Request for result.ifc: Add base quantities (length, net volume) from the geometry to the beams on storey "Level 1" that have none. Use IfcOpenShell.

First a look at what the model holds.

```python
import ifcopenshell
import ifcopenshell.util.element
import ifcopenshell.util.unit

model = ifcopenshell.open("result.ifc")
print(model.schema)
for unit_type in ("LENGTHUNIT", "AREAUNIT", "VOLUMEUNIT"):
    print(unit_type, ifcopenshell.util.unit.calculate_unit_scale(model, unit_type))
storey = next(s for s in model.by_type("IfcBuildingStorey") if s.Name == "Level 1")
beams = [e for e in ifcopenshell.util.element.get_decomposition(storey) if e.is_a("IfcBeam")]
for e in sorted(beams, key=lambda e: e.id()):
    print(e.id(), e.is_a(), e.Name, list(ifcopenshell.util.element.get_psets(e, qtos_only=True)), sep=" | ")
```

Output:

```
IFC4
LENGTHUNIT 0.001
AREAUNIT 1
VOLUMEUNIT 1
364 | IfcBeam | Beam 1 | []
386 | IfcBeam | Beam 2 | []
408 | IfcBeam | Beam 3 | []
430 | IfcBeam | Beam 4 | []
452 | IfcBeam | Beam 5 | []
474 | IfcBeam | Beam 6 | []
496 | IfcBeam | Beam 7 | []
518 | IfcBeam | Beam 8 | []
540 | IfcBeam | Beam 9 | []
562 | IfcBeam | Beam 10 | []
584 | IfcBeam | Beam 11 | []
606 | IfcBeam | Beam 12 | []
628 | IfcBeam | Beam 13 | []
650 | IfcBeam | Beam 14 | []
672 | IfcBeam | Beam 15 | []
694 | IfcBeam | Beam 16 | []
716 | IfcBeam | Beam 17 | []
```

```python
import ifcopenshell
import ifcopenshell.api.pset
import ifcopenshell.geom
import ifcopenshell.util.element
import ifcopenshell.util.shape
import ifcopenshell.util.unit

model = ifcopenshell.open("result.ifc")
unit_scale = ifcopenshell.util.unit.calculate_unit_scale(model)
volume_scale = ifcopenshell.util.unit.calculate_unit_scale(model, "VOLUMEUNIT")
settings = ifcopenshell.geom.settings()

storey = next(s for s in model.by_type("IfcBuildingStorey") if s.Name == "Level 1")
beams = [e for e in ifcopenshell.util.element.get_decomposition(storey) if e.is_a("IfcBeam")]

for e in sorted(beams, key=lambda e: e.id()):
    if ifcopenshell.util.element.get_psets(e, qtos_only=True, should_inherit=False):
        continue
    # Geometry comes back in metres, in the element's own axes.
    shape = ifcopenshell.geom.create_shape(settings, e)
    values = {
        "Length": ifcopenshell.util.shape.get_max_xyz(shape.geometry) / unit_scale,
        "NetVolume": ifcopenshell.util.shape.get_volume(shape.geometry) / volume_scale,
    }
    qto = ifcopenshell.api.pset.add_qto(model, product=e, name="Qto_BeamBaseQuantities")
    ifcopenshell.api.pset.edit_qto(model, qto=qto, properties=values)
    print(e.id(), {k: round(v, 3) for k, v in values.items()})

model.write("result_updated.ifc")
```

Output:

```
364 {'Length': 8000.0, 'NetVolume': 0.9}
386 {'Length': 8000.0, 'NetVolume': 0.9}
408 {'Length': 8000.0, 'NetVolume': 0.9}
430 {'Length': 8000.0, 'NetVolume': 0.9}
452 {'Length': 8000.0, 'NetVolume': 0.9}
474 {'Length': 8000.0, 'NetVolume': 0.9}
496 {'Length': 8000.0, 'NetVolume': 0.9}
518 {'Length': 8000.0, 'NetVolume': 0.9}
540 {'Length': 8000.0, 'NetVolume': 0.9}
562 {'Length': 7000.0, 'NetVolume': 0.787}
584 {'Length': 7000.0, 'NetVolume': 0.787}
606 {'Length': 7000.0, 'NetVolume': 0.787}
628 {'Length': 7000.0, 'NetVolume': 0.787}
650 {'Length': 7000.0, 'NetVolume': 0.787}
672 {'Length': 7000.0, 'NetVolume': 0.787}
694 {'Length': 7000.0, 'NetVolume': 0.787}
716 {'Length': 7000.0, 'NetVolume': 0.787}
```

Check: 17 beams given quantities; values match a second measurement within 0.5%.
